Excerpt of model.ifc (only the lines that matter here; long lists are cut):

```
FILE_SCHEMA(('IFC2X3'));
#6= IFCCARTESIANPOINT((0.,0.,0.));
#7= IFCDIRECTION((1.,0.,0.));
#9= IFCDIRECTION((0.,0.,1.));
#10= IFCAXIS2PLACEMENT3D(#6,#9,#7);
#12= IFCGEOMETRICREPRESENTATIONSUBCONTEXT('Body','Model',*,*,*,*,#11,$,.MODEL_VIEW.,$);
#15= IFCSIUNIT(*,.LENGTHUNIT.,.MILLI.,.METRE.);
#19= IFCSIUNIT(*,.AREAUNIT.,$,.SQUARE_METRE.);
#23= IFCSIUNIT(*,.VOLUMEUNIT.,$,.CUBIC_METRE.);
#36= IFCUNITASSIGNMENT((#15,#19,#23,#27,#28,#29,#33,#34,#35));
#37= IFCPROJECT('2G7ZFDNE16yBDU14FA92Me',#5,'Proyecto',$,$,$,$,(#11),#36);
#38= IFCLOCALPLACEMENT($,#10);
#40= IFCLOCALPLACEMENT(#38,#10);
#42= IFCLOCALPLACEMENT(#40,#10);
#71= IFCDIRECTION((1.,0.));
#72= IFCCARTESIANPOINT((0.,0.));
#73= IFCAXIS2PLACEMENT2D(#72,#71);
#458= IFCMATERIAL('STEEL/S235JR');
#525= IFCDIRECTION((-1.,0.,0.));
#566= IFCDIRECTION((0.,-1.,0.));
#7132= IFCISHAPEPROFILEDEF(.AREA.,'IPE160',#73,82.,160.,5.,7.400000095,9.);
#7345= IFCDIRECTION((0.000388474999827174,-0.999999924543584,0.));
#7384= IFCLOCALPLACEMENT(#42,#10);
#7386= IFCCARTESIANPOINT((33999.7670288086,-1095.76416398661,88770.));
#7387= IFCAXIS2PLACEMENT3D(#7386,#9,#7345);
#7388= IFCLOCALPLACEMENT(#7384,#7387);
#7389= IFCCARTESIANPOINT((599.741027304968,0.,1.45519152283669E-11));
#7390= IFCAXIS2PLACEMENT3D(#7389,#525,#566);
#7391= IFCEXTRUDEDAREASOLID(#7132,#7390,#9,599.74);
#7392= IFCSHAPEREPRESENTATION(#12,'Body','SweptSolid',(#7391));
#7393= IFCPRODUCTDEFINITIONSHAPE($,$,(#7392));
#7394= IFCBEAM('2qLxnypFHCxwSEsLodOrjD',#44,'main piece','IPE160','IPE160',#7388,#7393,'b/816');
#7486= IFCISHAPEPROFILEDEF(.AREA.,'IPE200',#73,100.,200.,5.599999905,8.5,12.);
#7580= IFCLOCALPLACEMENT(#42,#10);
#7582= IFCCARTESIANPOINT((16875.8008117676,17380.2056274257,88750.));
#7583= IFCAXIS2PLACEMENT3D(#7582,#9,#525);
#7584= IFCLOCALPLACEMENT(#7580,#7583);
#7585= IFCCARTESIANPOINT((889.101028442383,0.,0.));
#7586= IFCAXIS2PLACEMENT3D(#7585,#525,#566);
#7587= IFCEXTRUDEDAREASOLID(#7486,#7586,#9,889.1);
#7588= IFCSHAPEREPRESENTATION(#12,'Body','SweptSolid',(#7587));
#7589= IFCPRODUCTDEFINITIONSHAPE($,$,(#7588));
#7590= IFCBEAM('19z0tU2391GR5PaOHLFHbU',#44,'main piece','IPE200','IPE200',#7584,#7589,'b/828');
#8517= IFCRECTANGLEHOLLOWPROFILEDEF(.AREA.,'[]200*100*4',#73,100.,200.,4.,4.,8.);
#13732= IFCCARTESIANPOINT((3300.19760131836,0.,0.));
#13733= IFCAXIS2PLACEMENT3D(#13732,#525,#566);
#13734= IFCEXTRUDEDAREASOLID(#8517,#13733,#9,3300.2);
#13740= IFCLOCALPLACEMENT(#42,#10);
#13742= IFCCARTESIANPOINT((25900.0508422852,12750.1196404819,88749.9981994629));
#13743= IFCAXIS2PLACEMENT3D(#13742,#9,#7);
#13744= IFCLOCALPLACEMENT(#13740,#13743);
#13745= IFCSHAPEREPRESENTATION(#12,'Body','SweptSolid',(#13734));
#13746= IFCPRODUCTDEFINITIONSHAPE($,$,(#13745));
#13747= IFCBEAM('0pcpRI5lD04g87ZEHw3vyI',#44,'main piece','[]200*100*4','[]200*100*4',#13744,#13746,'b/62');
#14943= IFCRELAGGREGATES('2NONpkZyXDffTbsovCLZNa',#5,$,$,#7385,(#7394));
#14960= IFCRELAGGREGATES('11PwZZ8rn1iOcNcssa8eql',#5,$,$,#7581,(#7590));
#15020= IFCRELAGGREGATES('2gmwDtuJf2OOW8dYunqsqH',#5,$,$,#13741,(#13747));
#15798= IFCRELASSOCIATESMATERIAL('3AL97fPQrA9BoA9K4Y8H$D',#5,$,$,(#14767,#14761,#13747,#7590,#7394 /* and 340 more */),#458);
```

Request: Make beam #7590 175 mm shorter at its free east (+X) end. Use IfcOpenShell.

```python
import ifcopenshell
import ifcopenshell.util.representation
import ifcopenshell.util.unit

model = ifcopenshell.open("model.ifc")
unit_scale = ifcopenshell.util.unit.calculate_unit_scale(model)

member = model.by_guid("19z0tU2391GR5PaOHLFHbU")
change = -0.175 / unit_scale

# The extrusion runs towards the end named, so only its depth changes.
body = ifcopenshell.util.representation.get_representation(member, "Model", "Body")
solid = body.Items[0]
old_length = solid.Depth
solid.Depth += change

print(f"length {old_length:g} -> {solid.Depth:g}")

model.write("model_edited.ifc")
```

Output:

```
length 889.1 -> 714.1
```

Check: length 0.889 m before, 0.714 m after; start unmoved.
